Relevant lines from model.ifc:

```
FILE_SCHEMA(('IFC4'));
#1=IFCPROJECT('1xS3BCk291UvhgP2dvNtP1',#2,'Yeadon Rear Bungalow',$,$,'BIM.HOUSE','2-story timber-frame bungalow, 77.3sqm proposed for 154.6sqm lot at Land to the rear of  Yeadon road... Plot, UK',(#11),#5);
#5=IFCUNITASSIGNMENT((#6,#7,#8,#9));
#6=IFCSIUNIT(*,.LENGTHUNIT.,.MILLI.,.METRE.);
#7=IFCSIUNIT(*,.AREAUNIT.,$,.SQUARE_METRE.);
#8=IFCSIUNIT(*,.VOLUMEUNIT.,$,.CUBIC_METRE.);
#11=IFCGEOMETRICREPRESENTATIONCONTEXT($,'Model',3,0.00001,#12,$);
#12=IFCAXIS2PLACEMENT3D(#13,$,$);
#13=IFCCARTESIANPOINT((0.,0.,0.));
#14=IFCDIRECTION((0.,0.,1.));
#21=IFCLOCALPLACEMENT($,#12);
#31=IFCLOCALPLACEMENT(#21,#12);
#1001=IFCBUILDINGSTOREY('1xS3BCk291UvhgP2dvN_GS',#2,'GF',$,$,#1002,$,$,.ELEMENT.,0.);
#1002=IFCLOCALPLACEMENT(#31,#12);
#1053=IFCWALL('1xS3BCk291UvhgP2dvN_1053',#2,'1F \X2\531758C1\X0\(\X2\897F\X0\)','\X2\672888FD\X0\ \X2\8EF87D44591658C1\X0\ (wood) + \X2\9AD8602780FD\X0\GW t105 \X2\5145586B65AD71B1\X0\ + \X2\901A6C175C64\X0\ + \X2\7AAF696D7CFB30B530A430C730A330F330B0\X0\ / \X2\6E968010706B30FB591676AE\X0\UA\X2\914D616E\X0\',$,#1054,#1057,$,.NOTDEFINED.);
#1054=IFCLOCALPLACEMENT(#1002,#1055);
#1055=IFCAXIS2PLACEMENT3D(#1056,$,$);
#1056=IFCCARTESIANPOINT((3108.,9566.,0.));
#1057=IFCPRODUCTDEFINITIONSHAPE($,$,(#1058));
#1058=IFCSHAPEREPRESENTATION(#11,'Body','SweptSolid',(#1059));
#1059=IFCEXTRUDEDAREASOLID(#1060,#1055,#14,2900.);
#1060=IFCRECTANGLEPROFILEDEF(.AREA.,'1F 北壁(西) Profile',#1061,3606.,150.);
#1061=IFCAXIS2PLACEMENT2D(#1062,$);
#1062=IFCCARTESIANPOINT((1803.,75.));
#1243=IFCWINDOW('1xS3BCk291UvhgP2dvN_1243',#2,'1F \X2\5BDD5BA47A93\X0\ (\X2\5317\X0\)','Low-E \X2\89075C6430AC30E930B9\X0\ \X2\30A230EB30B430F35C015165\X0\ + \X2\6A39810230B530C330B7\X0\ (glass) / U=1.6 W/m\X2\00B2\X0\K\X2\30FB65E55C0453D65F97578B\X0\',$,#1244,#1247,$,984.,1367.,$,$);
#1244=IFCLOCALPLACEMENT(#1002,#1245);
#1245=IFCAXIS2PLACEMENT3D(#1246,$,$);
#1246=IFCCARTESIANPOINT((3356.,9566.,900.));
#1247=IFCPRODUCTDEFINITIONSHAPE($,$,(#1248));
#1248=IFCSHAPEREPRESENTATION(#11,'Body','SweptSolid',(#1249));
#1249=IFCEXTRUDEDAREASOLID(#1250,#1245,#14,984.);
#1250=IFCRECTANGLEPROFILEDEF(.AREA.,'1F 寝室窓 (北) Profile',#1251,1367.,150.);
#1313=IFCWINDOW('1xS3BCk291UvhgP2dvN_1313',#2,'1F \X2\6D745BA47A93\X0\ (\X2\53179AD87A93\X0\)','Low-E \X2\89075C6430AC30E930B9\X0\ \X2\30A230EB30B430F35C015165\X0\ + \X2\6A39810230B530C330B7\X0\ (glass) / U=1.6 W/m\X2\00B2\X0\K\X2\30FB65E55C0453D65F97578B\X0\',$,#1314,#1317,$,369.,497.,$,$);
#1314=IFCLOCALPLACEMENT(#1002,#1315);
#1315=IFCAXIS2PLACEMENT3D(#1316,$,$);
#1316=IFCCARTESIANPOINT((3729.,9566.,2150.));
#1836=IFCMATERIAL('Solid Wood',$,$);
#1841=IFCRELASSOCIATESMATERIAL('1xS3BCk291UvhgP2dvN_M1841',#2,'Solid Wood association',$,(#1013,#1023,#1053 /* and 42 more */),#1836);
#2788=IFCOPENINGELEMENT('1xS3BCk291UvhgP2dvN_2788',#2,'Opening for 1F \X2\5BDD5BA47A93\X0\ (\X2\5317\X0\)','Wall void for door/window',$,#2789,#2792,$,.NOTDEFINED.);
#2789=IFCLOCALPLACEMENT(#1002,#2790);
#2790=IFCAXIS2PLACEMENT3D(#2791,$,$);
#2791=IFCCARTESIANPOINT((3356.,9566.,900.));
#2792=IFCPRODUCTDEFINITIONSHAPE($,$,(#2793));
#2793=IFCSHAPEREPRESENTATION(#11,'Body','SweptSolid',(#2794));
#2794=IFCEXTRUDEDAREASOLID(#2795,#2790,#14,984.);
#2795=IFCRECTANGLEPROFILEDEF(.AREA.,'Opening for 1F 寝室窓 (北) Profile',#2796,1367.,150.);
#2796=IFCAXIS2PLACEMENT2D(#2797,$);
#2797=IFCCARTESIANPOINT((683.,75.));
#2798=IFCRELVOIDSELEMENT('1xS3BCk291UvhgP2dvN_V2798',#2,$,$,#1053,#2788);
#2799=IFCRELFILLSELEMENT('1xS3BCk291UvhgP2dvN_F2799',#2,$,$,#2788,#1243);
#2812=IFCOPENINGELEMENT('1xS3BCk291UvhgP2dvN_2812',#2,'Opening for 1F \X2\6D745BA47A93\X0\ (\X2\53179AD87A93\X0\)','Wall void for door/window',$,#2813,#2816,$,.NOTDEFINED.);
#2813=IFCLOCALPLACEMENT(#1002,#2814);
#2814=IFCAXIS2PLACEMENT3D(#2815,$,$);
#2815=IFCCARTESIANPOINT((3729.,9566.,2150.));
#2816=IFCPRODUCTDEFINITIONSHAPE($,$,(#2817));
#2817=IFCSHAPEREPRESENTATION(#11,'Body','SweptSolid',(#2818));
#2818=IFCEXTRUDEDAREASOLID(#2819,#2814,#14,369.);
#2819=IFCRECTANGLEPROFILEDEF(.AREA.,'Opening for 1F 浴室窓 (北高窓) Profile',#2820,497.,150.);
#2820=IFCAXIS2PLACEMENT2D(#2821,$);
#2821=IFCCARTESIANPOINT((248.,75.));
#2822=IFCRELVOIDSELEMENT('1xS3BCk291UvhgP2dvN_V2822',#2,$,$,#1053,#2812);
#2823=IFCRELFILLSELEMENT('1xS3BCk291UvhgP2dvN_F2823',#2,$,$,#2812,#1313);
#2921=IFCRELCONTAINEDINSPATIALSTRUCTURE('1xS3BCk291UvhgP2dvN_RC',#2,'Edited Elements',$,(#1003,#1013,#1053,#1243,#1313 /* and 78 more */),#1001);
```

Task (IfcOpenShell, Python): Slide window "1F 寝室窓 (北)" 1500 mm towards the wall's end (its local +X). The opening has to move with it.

```python
import ifcopenshell
import ifcopenshell.api.geometry
import ifcopenshell.util.placement

model = ifcopenshell.open("model.ifc")

window = model.by_id(1243)
opening = window.FillsVoids[0].RelatingOpeningElement
wall = opening.VoidsElements[0].RelatingBuildingElement

wall_matrix = ifcopenshell.util.placement.get_local_placement(wall.ObjectPlacement)
shift = wall_matrix[:3, 0] * 1500.0
before = ifcopenshell.util.placement.get_local_placement(window.ObjectPlacement)[:3, 3].copy()

# The window is not placed relative to its opening, so move both.
for product in (opening, window):
    matrix = ifcopenshell.util.placement.get_local_placement(product.ObjectPlacement)
    matrix[:3, 3] += shift
    ifcopenshell.api.geometry.edit_object_placement(model, product=product, matrix=matrix, is_si=False)

after = ifcopenshell.util.placement.get_local_placement(window.ObjectPlacement)[:3, 3]
print("window moved by", (after - before).round(3) + 0.0)

model.write("model_v2.ifc")
```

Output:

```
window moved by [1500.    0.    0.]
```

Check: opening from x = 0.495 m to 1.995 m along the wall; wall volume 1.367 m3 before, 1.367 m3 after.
